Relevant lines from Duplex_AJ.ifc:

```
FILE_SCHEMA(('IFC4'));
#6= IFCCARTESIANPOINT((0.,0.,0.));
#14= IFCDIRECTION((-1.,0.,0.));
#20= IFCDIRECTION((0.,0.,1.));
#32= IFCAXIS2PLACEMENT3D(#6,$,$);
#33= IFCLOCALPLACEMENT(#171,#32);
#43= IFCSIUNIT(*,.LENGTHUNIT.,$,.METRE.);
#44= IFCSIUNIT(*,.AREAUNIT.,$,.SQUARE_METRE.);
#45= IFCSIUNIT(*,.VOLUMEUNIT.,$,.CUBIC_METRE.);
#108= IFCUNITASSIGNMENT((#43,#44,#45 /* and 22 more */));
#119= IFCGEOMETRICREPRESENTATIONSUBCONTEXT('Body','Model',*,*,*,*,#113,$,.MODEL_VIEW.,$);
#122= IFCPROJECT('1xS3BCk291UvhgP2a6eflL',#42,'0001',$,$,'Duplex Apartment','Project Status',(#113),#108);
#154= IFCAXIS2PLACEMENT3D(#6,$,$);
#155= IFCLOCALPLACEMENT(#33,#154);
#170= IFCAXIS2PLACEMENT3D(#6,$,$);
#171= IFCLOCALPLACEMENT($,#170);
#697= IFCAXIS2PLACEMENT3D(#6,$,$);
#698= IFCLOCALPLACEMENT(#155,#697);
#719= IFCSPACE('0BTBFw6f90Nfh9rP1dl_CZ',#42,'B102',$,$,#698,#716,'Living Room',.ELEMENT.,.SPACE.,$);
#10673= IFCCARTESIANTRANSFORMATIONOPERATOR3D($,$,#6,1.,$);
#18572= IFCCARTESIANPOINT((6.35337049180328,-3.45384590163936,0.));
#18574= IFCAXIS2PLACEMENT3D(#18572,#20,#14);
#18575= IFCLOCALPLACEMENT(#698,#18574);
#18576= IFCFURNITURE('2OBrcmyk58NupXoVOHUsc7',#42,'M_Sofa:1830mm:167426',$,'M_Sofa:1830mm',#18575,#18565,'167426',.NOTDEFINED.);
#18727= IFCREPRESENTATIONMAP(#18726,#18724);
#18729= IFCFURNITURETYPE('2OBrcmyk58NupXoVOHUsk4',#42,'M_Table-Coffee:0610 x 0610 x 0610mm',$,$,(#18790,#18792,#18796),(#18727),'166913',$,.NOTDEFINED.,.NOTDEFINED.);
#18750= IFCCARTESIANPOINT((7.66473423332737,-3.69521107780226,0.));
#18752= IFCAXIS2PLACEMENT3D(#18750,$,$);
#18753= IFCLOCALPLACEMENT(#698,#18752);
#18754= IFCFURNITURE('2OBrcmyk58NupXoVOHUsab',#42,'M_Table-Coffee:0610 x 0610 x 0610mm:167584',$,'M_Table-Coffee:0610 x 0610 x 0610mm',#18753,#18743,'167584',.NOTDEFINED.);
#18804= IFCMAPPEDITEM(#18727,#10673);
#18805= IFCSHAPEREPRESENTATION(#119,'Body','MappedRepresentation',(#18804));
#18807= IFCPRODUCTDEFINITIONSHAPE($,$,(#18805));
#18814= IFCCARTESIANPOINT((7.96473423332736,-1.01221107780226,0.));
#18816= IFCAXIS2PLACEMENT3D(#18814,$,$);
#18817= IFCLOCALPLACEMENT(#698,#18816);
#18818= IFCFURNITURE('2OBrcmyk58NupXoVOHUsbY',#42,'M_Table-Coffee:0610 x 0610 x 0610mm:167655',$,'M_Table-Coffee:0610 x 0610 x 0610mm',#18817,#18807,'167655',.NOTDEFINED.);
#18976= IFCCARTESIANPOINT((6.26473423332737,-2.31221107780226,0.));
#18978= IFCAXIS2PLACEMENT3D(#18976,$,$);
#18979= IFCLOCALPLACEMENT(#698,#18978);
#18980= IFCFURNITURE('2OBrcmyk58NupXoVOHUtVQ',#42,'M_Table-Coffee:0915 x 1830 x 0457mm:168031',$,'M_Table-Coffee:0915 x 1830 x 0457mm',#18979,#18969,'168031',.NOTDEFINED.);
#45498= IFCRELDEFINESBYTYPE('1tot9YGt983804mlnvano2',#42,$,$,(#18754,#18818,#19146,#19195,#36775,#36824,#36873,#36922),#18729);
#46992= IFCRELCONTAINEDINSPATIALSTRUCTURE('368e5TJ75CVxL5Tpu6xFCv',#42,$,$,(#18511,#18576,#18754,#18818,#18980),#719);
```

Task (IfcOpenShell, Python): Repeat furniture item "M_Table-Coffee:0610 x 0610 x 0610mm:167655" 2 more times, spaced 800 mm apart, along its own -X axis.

```python
import ifcopenshell
import ifcopenshell.api.geometry
import ifcopenshell.api.root
import ifcopenshell.util.element
import ifcopenshell.util.placement

model = ifcopenshell.open("Duplex_AJ.ifc")


def reuse_history(source, copy):
    """copy_class also copies each property set's owner history, people and application; keep the originals."""
    for rel in copy.IsDefinedBy:
        if rel.is_a("IfcRelDefinesByProperties") and (history := rel.RelatingPropertyDefinition.OwnerHistory):
            rel.RelatingPropertyDefinition.OwnerHistory = source.OwnerHistory
            ifcopenshell.util.element.remove_deep2(model, history)


source = model.by_id(18818)
base = ifcopenshell.util.placement.get_local_placement(source.ObjectPlacement)
step = -base[:3, 0] * 0.8

for i in range(1, 3):
    copy = ifcopenshell.api.root.copy_class(model, product=source)
    copy.Representation = ifcopenshell.util.element.copy_deep(
        model, source.Representation, exclude=["IfcGeometricRepresentationContext", "IfcRepresentationMap"]
    )
    copy.Name = "M_Table-Coffee:0610 x 0610 x 0610mm"
    copy.Tag = None
    reuse_history(source, copy)
    matrix = base.copy()
    matrix[:3, 3] += i * step
    print("added at", matrix[:3, 3].round(3) + 0.0)
    ifcopenshell.api.geometry.edit_object_placement(model, product=copy, matrix=matrix, is_si=False)

model.write("Duplex_AJ_v2.ifc")
```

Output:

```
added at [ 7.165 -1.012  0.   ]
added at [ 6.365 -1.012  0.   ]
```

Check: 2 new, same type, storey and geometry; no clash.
